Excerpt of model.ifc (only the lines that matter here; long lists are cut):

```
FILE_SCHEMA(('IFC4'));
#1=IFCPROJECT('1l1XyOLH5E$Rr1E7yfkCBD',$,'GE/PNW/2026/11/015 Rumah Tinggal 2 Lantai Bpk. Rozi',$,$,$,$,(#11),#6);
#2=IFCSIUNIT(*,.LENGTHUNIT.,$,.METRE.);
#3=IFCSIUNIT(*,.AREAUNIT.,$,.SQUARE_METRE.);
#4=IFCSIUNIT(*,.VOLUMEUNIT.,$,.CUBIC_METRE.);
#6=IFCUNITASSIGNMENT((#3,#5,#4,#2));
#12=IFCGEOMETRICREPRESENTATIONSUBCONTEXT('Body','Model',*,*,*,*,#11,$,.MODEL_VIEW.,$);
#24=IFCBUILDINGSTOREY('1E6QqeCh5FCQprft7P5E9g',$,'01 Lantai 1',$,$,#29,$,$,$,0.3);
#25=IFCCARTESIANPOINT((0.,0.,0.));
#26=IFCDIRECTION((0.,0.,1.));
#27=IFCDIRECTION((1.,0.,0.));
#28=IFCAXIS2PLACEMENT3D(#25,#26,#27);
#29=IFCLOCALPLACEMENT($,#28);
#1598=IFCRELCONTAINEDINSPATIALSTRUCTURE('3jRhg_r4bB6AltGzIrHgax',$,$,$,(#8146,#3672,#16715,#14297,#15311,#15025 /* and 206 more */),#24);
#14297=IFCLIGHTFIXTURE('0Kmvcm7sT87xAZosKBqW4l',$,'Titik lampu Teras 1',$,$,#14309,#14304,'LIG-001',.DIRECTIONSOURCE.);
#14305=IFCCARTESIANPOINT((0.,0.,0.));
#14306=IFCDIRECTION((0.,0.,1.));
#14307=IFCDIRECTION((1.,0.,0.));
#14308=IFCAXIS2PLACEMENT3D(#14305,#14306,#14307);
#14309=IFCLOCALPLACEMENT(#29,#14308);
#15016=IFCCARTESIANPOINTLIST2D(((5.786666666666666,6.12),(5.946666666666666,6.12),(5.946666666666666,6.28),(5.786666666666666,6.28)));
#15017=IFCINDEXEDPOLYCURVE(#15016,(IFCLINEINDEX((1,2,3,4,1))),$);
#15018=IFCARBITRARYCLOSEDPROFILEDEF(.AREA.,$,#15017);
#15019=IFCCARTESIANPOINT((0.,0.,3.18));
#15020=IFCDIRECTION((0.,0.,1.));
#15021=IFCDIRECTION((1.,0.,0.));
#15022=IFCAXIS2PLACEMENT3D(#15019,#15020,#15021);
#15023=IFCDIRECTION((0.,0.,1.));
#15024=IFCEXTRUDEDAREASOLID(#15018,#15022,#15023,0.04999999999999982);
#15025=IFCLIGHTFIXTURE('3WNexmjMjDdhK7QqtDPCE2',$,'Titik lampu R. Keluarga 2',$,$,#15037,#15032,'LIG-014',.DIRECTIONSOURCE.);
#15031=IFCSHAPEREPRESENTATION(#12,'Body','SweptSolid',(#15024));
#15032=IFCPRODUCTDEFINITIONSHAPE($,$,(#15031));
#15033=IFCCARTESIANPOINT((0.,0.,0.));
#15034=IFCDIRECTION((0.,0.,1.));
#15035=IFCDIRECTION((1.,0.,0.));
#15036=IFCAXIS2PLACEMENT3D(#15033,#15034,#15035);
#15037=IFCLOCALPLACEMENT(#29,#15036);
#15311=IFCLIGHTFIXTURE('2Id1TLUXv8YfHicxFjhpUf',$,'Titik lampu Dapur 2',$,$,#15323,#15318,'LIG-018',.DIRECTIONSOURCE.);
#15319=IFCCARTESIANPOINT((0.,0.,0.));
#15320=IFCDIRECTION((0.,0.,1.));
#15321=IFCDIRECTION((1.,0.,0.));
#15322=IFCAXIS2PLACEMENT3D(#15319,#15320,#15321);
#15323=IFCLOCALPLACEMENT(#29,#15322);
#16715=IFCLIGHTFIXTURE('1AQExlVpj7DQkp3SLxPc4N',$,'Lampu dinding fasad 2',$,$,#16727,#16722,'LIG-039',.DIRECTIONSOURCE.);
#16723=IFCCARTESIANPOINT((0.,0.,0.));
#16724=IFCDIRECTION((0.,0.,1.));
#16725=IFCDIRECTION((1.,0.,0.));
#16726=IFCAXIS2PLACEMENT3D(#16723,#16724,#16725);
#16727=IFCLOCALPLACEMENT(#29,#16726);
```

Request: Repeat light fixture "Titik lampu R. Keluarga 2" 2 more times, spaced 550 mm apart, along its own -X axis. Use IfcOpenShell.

```python
import ifcopenshell
import ifcopenshell.api.geometry
import ifcopenshell.api.root
import ifcopenshell.util.element
import ifcopenshell.util.placement
import ifcopenshell.util.unit

model = ifcopenshell.open("model.ifc")
unit_scale = ifcopenshell.util.unit.calculate_unit_scale(model)

source = model.by_guid("3WNexmjMjDdhK7QqtDPCE2")
base = ifcopenshell.util.placement.get_local_placement(source.ObjectPlacement)
step = -base[:3, 0] * 0.55 / unit_scale

for i in range(1, 3):
    copy = ifcopenshell.api.root.copy_class(model, product=source)
    copy.Representation = ifcopenshell.util.element.copy_deep(
        model, source.Representation, exclude=["IfcGeometricRepresentationContext", "IfcRepresentationMap"]
    )
    copy.Tag = None
    matrix = base.copy()
    matrix[:3, 3] += i * step
    print("added at", matrix[:3, 3].round(3) + 0.0)
    ifcopenshell.api.geometry.edit_object_placement(model, product=copy, matrix=matrix, is_si=False)

model.write("model_edited.ifc")
```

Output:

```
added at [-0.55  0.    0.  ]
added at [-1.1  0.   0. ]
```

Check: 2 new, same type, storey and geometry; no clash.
